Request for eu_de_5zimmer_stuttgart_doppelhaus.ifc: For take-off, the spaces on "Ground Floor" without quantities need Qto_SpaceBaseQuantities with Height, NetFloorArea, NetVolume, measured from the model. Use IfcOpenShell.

First a look at what the model holds.

```python
import ifcopenshell
import ifcopenshell.util.element
import ifcopenshell.util.unit

model = ifcopenshell.open("eu_de_5zimmer_stuttgart_doppelhaus.ifc")
print(model.schema)
for unit_type in ("LENGTHUNIT", "AREAUNIT", "VOLUMEUNIT"):
    print(unit_type, ifcopenshell.util.unit.calculate_unit_scale(model, unit_type))
storey = next(s for s in model.by_type("IfcBuildingStorey") if s.Name == "Ground Floor")
spaces = [e for e in ifcopenshell.util.element.get_decomposition(storey) if e.is_a("IfcSpace")]
for e in sorted(spaces, key=lambda e: e.id()):
    print(e.id(), e.is_a(), e.Name, list(ifcopenshell.util.element.get_psets(e, qtos_only=True)), sep=" | ")
```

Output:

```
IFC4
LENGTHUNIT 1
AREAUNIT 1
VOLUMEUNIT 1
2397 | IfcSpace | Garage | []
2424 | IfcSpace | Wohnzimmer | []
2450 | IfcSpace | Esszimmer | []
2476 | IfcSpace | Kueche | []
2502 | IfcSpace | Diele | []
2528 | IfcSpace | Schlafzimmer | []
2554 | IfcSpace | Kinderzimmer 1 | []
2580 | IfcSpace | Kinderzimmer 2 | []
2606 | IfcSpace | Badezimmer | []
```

```python
import ifcopenshell
import ifcopenshell.api.pset
import ifcopenshell.geom
import ifcopenshell.util.element
import ifcopenshell.util.shape
import ifcopenshell.util.unit

model = ifcopenshell.open("eu_de_5zimmer_stuttgart_doppelhaus.ifc")
unit_scale = ifcopenshell.util.unit.calculate_unit_scale(model)
area_scale = ifcopenshell.util.unit.calculate_unit_scale(model, "AREAUNIT")
volume_scale = ifcopenshell.util.unit.calculate_unit_scale(model, "VOLUMEUNIT")
settings = ifcopenshell.geom.settings()

storey = next(s for s in model.by_type("IfcBuildingStorey") if s.Name == "Ground Floor")
spaces = [e for e in ifcopenshell.util.element.get_decomposition(storey) if e.is_a("IfcSpace")]

for e in sorted(spaces, key=lambda e: e.id()):
    if ifcopenshell.util.element.get_psets(e, qtos_only=True, should_inherit=False):
        continue
    # Geometry comes back in metres, in the element's own axes.
    shape = ifcopenshell.geom.create_shape(settings, e)
    values = {
        "Height": ifcopenshell.util.shape.get_z(shape.geometry) / unit_scale,
        "NetFloorArea": ifcopenshell.util.shape.get_footprint_area(shape.geometry) / area_scale,
        "NetVolume": ifcopenshell.util.shape.get_volume(shape.geometry) / volume_scale,
    }
    qto = ifcopenshell.api.pset.add_qto(model, product=e, name="Qto_SpaceBaseQuantities")
    ifcopenshell.api.pset.edit_qto(model, qto=qto, properties=values)
    print(e.id(), {k: round(v, 3) for k, v in values.items()})

model.write("eu_de_5zimmer_stuttgart_doppelhaus_rev.ifc")
```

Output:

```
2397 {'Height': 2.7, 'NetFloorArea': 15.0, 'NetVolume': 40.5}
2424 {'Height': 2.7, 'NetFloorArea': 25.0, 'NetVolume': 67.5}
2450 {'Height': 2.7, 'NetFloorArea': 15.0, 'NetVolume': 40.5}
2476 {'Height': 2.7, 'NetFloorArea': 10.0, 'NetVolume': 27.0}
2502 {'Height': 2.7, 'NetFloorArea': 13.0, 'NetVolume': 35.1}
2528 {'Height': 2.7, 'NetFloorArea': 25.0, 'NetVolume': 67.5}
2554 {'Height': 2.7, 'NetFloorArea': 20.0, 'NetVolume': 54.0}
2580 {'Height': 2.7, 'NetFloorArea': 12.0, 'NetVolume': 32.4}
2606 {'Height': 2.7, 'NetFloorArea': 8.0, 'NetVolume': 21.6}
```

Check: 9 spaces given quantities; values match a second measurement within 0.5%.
